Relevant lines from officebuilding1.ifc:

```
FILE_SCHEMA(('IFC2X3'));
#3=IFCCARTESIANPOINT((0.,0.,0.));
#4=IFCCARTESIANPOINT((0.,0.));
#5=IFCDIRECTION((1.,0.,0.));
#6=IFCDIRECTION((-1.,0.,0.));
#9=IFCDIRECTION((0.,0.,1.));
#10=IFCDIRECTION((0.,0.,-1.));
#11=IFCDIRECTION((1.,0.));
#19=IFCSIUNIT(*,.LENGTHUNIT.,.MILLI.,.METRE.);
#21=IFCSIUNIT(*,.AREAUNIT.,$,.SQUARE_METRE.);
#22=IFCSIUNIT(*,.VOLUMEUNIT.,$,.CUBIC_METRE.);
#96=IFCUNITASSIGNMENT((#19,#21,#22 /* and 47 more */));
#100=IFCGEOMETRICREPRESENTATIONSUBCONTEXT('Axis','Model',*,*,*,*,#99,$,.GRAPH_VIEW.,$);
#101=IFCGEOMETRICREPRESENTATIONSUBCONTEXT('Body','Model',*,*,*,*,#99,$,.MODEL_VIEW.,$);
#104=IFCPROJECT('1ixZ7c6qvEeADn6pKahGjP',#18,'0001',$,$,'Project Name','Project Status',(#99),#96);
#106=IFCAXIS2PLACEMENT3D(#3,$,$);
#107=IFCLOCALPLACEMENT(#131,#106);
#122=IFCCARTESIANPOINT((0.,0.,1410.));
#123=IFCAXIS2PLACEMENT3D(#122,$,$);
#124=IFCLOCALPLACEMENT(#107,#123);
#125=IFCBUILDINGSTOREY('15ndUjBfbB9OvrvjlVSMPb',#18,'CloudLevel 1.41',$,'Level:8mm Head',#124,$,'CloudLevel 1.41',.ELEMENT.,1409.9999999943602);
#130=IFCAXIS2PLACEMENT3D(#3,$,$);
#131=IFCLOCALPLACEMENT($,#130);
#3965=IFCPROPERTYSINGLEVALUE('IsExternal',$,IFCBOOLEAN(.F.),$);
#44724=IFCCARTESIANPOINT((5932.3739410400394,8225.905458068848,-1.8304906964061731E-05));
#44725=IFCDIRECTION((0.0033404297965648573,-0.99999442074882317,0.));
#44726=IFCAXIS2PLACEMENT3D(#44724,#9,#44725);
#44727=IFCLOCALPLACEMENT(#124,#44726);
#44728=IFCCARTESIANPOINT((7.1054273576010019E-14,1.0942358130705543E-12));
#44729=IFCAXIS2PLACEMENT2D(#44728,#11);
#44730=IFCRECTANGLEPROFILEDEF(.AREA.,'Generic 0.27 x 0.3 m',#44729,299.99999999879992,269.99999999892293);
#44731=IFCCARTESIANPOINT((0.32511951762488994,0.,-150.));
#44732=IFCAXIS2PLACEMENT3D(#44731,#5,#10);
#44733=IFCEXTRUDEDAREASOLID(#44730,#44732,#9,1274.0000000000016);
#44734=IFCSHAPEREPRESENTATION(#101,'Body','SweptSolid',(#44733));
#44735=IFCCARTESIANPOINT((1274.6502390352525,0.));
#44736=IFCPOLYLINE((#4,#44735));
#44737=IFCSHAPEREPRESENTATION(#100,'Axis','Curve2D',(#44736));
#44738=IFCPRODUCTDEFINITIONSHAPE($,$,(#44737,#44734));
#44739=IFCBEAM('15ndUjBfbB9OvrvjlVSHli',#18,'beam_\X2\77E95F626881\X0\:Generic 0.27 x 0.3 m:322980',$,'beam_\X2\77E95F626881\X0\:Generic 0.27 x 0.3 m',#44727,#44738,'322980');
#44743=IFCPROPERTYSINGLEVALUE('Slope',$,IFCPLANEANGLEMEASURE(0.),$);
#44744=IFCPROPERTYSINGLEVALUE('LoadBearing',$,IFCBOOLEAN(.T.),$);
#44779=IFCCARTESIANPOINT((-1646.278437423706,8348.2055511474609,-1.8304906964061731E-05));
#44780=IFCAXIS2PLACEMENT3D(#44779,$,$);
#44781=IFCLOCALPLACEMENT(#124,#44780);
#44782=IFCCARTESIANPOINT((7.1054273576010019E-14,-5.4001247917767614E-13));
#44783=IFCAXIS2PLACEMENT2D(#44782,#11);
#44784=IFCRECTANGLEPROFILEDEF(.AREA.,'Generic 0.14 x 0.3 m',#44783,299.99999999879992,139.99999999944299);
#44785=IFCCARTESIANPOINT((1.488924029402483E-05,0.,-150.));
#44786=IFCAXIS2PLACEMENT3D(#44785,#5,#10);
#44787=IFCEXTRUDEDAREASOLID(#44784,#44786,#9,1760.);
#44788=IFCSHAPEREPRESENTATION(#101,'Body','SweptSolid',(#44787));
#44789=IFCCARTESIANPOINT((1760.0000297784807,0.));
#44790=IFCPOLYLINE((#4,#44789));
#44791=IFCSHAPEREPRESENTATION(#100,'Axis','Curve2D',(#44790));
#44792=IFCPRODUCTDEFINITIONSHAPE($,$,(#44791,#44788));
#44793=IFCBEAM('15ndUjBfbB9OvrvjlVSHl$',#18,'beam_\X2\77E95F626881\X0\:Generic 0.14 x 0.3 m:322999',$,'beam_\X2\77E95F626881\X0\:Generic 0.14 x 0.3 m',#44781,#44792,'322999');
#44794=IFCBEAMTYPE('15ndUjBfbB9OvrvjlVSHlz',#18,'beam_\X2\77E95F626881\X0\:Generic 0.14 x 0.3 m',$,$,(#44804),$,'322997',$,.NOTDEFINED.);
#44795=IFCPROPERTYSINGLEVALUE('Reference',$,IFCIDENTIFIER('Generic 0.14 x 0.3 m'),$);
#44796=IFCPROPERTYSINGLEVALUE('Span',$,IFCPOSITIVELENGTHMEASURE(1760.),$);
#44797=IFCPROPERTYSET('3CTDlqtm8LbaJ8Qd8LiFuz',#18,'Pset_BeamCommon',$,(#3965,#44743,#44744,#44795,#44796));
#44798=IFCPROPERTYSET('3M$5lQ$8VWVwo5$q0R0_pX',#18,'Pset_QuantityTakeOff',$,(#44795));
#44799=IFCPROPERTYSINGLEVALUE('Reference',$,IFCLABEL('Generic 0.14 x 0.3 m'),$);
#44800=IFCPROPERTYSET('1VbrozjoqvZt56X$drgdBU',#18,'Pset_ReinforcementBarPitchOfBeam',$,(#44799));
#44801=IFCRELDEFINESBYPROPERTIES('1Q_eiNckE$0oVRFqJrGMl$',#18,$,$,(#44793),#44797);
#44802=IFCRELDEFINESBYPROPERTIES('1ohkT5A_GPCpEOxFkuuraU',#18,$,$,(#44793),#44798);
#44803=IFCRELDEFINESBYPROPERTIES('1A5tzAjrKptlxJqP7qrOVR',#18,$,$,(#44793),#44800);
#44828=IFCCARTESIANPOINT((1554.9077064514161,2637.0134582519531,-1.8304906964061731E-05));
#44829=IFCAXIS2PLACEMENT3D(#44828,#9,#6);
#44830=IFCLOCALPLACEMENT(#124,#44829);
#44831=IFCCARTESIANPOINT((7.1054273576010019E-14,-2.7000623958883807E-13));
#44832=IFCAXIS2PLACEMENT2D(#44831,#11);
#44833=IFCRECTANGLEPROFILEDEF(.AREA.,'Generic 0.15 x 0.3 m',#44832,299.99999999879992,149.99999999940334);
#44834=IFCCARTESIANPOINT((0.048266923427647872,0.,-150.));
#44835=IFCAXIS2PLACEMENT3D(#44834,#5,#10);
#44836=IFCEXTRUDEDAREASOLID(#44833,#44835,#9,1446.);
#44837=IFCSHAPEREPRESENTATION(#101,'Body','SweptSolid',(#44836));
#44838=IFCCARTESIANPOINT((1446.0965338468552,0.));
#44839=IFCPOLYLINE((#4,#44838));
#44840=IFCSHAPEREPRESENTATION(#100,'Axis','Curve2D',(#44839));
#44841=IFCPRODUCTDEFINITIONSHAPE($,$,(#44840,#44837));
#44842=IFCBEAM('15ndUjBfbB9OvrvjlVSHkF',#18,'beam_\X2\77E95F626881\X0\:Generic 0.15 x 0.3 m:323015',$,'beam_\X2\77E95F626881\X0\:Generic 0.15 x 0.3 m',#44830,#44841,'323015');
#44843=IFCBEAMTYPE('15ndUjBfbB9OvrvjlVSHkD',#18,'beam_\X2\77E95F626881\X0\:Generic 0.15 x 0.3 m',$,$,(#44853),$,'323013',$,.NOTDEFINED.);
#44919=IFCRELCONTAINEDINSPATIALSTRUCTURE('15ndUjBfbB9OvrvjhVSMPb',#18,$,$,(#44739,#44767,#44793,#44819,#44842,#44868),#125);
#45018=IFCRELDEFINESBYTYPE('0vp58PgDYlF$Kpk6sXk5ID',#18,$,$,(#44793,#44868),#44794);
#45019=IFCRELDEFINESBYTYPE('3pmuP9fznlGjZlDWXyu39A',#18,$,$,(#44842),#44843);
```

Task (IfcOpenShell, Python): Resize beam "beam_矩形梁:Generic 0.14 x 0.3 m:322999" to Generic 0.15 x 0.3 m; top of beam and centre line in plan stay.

```python
import ifcopenshell
import ifcopenshell.api.pset
import ifcopenshell.api.type
import ifcopenshell.util.element
import ifcopenshell.util.representation

model = ifcopenshell.open("officebuilding1.ifc")

member = model.by_guid("15ndUjBfbB9OvrvjlVSHl$")
source = next(p for p in model.by_type("IfcRectangleProfileDef") if p.ProfileName == "Generic 0.15 x 0.3 m")

body = ifcopenshell.util.representation.get_representation(member, "Model", "Body")
solid = body.Items[0]
old_profile = solid.SweptArea

# Copy the section's sizes but keep this member's own profile position.
profile = ifcopenshell.util.element.copy(model, source)
# Profiles are centred, so shift by half the change in depth to hold the top.
shift = (old_profile.XDim - profile.XDim) / 2
x, y = old_profile.Position.Location.Coordinates
up = (-1.0, 0.0)  # upwards, in the solid's own plane
location = model.createIfcCartesianPoint((x + up[0] * shift, y + up[1] * shift))
profile.Position = model.createIfcAxis2Placement2D(location, old_profile.Position.RefDirection)
solid.SweptArea = profile
if not model.get_total_inverses(old_profile):
    ifcopenshell.util.element.remove_deep2(model, old_profile)

new_type = model.by_guid("15ndUjBfbB9OvrvjlVSHkD")
ifcopenshell.api.type.assign_type(
    model, related_objects=[member], relating_type=new_type, should_map_representations=False
)
member.Name = member.Name.replace("Generic 0.14 x 0.3 m", "Generic 0.15 x 0.3 m")
member.ObjectType = "beam_矩形梁:Generic 0.15 x 0.3 m"
pset = model.by_id(ifcopenshell.util.element.get_pset(member, "Pset_BeamCommon", should_inherit=False)["id"])
ifcopenshell.api.pset.edit_pset(model, pset=pset, properties={"Reference": "Generic 0.15 x 0.3 m"})
pset = model.by_id(ifcopenshell.util.element.get_pset(member, "Pset_QuantityTakeOff", should_inherit=False)["id"])
ifcopenshell.api.pset.edit_pset(model, pset=pset, properties={"Reference": "Generic 0.15 x 0.3 m"})
pset = model.by_id(ifcopenshell.util.element.get_pset(member, "Pset_ReinforcementBarPitchOfBeam", should_inherit=False)["id"])
ifcopenshell.api.pset.edit_pset(model, pset=pset, properties={"Reference": "Generic 0.15 x 0.3 m"})

print(solid.SweptArea)

model.write("officebuilding1_edited.ifc")
```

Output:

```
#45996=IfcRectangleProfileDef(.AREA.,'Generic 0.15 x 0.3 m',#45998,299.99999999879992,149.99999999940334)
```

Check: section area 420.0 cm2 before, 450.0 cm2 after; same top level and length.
